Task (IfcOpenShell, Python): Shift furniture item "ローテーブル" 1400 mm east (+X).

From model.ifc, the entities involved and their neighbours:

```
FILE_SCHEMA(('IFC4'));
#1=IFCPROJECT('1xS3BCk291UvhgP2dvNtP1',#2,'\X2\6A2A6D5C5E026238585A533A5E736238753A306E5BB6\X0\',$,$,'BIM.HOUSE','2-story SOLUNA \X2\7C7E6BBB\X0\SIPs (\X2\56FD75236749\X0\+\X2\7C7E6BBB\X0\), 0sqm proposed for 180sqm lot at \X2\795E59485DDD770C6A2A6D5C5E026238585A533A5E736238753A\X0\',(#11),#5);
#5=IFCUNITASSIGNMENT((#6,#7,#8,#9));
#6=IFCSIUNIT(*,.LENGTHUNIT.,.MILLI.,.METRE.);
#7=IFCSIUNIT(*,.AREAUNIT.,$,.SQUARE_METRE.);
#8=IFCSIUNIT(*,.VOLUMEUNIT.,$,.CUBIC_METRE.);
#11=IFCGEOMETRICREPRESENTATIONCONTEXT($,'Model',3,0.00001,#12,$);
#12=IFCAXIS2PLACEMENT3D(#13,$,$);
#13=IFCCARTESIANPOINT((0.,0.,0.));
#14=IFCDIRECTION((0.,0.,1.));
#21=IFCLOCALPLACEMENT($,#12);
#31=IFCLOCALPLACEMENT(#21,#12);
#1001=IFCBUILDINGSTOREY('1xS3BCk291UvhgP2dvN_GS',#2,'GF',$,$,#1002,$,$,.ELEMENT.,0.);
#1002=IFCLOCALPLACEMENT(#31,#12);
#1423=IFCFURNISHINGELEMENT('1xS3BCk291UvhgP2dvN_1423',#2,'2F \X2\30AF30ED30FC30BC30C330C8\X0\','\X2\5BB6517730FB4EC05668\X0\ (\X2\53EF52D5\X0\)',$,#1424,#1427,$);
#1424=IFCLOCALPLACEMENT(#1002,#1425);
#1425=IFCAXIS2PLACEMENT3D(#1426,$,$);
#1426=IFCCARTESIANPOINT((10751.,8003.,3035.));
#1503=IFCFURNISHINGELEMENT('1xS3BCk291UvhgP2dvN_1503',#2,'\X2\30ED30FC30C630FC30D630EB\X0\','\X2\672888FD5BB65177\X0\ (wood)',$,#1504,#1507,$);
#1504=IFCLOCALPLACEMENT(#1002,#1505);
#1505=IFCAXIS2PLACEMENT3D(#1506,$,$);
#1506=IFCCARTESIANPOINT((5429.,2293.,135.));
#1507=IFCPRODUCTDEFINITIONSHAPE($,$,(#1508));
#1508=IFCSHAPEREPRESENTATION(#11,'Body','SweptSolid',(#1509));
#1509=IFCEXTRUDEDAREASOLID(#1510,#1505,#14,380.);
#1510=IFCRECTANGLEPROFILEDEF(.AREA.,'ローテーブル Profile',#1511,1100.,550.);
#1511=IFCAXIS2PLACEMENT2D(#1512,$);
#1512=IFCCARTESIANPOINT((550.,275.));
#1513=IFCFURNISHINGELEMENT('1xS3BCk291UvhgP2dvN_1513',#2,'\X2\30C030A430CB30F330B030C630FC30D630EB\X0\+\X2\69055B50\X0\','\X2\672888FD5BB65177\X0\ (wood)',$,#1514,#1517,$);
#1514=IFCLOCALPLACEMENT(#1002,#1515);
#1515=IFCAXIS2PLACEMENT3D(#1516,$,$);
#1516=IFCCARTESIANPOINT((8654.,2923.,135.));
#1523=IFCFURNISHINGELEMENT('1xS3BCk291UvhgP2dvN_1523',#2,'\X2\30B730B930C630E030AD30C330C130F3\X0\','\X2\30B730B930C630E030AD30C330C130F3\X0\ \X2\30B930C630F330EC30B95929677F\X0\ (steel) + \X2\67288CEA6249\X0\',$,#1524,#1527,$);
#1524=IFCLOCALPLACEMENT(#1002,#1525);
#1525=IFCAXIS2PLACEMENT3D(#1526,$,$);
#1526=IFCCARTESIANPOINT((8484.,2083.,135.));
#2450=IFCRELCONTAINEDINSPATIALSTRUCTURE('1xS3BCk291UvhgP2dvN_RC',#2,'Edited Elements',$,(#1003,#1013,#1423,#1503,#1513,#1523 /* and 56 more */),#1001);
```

```python
import ifcopenshell
import ifcopenshell.api.geometry
import ifcopenshell.util.placement
import ifcopenshell.util.unit

model = ifcopenshell.open("model.ifc")
unit_scale = ifcopenshell.util.unit.calculate_unit_scale(model)

item = model.by_id(1503)
matrix = ifcopenshell.util.placement.get_local_placement(item.ObjectPlacement)
matrix[0, 3] += 1.4 / unit_scale
ifcopenshell.api.geometry.edit_object_placement(model, product=item, matrix=matrix, is_si=False)

print(ifcopenshell.util.placement.get_local_placement(item.ObjectPlacement).round(3) + 0.0)

model.write("model_rev.ifc")
```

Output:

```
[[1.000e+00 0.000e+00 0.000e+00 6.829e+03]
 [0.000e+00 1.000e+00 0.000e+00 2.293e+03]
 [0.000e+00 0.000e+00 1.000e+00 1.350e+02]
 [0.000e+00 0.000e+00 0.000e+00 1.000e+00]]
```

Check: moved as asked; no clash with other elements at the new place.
